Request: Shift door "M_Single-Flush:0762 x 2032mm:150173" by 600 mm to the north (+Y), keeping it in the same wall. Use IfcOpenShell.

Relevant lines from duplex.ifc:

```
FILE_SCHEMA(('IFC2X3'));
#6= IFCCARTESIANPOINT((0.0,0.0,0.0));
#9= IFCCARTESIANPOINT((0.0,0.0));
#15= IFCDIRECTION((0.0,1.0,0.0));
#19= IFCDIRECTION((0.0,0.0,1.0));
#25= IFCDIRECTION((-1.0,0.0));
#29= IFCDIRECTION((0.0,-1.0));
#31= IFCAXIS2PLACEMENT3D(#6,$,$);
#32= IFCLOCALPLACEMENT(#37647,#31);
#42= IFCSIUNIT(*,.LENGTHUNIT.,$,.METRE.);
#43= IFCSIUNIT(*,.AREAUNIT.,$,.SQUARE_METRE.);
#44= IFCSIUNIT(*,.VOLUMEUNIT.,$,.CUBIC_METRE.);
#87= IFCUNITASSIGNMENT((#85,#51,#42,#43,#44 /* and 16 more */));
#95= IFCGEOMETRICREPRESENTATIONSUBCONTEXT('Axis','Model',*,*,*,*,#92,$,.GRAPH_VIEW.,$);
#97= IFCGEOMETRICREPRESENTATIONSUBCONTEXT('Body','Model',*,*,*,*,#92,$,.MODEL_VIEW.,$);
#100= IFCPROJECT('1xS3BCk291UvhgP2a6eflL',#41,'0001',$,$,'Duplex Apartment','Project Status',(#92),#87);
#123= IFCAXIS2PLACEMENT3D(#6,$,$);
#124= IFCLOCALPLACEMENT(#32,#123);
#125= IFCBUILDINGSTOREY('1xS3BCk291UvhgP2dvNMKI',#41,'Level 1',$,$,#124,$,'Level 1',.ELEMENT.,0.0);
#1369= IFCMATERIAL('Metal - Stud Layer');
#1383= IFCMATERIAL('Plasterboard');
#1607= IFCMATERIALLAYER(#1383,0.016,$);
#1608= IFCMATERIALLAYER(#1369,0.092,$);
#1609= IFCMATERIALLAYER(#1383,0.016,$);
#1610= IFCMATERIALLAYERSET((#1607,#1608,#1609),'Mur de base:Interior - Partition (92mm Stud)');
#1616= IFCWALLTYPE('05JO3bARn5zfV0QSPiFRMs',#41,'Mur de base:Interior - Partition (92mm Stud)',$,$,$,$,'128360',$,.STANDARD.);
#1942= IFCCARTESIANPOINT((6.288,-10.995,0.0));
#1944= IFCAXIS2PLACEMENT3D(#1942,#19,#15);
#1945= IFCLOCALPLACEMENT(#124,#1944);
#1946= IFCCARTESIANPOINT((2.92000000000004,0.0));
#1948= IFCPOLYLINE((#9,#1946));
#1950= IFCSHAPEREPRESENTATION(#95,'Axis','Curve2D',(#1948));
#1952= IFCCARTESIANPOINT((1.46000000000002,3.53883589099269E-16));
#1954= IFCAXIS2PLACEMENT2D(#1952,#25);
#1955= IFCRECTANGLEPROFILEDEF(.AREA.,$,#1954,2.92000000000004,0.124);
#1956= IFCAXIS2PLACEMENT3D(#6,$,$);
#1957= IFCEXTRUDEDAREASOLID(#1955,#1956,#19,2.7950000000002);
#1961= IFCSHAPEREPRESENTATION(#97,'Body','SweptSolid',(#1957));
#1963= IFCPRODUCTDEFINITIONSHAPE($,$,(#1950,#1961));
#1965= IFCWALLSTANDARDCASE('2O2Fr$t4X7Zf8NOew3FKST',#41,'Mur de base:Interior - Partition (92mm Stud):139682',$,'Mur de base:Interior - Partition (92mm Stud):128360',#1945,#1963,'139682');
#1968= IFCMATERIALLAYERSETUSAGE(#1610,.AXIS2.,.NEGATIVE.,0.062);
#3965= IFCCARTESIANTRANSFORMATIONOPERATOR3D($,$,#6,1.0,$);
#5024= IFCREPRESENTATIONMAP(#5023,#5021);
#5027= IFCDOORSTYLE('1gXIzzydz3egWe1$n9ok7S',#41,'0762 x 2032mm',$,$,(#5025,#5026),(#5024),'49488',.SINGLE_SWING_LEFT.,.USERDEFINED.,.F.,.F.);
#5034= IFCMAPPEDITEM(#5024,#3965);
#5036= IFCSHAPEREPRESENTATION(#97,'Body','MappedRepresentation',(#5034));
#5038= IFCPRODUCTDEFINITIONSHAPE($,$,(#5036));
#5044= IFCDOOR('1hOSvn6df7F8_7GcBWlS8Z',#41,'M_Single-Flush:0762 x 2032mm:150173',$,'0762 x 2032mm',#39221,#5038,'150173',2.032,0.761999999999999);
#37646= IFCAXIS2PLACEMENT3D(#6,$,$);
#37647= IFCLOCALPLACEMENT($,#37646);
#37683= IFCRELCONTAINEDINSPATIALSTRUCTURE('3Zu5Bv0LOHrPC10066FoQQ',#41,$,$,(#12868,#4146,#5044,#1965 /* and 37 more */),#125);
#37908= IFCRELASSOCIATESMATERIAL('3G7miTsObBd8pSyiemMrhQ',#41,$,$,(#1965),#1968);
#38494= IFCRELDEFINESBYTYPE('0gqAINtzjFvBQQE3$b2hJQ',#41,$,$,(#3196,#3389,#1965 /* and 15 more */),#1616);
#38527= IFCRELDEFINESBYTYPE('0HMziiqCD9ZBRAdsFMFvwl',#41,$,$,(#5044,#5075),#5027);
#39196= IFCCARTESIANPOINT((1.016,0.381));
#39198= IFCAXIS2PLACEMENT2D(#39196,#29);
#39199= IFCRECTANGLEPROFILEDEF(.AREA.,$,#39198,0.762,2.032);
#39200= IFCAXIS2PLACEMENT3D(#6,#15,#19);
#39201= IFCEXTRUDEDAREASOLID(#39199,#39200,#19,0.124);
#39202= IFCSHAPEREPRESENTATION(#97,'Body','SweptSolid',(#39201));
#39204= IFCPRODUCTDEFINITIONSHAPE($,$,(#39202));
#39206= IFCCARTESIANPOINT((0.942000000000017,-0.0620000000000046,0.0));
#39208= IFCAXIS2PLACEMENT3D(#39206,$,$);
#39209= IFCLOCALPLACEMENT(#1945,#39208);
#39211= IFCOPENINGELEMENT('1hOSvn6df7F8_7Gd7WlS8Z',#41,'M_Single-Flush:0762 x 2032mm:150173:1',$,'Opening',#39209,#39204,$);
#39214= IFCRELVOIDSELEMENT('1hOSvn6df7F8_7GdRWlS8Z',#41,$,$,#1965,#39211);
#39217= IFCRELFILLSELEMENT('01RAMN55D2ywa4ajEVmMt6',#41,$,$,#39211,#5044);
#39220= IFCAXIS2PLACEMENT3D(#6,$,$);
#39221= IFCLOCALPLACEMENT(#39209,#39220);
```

```python
import ifcopenshell
import ifcopenshell.api.geometry
import ifcopenshell.util.placement
import ifcopenshell.util.unit

model = ifcopenshell.open("duplex.ifc")
unit_scale = ifcopenshell.util.unit.calculate_unit_scale(model)

door = model.by_guid("1hOSvn6df7F8_7GcBWlS8Z")
opening = door.FillsVoids[0].RelatingOpeningElement
wall = opening.VoidsElements[0].RelatingBuildingElement

wall_matrix = ifcopenshell.util.placement.get_local_placement(wall.ObjectPlacement)
shift = wall_matrix[:3, 0] * 0.6 / unit_scale
before = ifcopenshell.util.placement.get_local_placement(door.ObjectPlacement)[:3, 3].copy()

# The door is placed relative to its opening, so it follows when the opening moves.
matrix = ifcopenshell.util.placement.get_local_placement(opening.ObjectPlacement)
matrix[:3, 3] += shift
ifcopenshell.api.geometry.edit_object_placement(
    model, product=opening, matrix=matrix, is_si=False, should_transform_children=True
)

after = ifcopenshell.util.placement.get_local_placement(door.ObjectPlacement)[:3, 3]
print("door moved by", (after - before).round(3) + 0.0)

model.write("duplex_v2.ifc")
```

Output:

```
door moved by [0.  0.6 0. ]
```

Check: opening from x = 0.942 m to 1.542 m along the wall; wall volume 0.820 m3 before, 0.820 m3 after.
